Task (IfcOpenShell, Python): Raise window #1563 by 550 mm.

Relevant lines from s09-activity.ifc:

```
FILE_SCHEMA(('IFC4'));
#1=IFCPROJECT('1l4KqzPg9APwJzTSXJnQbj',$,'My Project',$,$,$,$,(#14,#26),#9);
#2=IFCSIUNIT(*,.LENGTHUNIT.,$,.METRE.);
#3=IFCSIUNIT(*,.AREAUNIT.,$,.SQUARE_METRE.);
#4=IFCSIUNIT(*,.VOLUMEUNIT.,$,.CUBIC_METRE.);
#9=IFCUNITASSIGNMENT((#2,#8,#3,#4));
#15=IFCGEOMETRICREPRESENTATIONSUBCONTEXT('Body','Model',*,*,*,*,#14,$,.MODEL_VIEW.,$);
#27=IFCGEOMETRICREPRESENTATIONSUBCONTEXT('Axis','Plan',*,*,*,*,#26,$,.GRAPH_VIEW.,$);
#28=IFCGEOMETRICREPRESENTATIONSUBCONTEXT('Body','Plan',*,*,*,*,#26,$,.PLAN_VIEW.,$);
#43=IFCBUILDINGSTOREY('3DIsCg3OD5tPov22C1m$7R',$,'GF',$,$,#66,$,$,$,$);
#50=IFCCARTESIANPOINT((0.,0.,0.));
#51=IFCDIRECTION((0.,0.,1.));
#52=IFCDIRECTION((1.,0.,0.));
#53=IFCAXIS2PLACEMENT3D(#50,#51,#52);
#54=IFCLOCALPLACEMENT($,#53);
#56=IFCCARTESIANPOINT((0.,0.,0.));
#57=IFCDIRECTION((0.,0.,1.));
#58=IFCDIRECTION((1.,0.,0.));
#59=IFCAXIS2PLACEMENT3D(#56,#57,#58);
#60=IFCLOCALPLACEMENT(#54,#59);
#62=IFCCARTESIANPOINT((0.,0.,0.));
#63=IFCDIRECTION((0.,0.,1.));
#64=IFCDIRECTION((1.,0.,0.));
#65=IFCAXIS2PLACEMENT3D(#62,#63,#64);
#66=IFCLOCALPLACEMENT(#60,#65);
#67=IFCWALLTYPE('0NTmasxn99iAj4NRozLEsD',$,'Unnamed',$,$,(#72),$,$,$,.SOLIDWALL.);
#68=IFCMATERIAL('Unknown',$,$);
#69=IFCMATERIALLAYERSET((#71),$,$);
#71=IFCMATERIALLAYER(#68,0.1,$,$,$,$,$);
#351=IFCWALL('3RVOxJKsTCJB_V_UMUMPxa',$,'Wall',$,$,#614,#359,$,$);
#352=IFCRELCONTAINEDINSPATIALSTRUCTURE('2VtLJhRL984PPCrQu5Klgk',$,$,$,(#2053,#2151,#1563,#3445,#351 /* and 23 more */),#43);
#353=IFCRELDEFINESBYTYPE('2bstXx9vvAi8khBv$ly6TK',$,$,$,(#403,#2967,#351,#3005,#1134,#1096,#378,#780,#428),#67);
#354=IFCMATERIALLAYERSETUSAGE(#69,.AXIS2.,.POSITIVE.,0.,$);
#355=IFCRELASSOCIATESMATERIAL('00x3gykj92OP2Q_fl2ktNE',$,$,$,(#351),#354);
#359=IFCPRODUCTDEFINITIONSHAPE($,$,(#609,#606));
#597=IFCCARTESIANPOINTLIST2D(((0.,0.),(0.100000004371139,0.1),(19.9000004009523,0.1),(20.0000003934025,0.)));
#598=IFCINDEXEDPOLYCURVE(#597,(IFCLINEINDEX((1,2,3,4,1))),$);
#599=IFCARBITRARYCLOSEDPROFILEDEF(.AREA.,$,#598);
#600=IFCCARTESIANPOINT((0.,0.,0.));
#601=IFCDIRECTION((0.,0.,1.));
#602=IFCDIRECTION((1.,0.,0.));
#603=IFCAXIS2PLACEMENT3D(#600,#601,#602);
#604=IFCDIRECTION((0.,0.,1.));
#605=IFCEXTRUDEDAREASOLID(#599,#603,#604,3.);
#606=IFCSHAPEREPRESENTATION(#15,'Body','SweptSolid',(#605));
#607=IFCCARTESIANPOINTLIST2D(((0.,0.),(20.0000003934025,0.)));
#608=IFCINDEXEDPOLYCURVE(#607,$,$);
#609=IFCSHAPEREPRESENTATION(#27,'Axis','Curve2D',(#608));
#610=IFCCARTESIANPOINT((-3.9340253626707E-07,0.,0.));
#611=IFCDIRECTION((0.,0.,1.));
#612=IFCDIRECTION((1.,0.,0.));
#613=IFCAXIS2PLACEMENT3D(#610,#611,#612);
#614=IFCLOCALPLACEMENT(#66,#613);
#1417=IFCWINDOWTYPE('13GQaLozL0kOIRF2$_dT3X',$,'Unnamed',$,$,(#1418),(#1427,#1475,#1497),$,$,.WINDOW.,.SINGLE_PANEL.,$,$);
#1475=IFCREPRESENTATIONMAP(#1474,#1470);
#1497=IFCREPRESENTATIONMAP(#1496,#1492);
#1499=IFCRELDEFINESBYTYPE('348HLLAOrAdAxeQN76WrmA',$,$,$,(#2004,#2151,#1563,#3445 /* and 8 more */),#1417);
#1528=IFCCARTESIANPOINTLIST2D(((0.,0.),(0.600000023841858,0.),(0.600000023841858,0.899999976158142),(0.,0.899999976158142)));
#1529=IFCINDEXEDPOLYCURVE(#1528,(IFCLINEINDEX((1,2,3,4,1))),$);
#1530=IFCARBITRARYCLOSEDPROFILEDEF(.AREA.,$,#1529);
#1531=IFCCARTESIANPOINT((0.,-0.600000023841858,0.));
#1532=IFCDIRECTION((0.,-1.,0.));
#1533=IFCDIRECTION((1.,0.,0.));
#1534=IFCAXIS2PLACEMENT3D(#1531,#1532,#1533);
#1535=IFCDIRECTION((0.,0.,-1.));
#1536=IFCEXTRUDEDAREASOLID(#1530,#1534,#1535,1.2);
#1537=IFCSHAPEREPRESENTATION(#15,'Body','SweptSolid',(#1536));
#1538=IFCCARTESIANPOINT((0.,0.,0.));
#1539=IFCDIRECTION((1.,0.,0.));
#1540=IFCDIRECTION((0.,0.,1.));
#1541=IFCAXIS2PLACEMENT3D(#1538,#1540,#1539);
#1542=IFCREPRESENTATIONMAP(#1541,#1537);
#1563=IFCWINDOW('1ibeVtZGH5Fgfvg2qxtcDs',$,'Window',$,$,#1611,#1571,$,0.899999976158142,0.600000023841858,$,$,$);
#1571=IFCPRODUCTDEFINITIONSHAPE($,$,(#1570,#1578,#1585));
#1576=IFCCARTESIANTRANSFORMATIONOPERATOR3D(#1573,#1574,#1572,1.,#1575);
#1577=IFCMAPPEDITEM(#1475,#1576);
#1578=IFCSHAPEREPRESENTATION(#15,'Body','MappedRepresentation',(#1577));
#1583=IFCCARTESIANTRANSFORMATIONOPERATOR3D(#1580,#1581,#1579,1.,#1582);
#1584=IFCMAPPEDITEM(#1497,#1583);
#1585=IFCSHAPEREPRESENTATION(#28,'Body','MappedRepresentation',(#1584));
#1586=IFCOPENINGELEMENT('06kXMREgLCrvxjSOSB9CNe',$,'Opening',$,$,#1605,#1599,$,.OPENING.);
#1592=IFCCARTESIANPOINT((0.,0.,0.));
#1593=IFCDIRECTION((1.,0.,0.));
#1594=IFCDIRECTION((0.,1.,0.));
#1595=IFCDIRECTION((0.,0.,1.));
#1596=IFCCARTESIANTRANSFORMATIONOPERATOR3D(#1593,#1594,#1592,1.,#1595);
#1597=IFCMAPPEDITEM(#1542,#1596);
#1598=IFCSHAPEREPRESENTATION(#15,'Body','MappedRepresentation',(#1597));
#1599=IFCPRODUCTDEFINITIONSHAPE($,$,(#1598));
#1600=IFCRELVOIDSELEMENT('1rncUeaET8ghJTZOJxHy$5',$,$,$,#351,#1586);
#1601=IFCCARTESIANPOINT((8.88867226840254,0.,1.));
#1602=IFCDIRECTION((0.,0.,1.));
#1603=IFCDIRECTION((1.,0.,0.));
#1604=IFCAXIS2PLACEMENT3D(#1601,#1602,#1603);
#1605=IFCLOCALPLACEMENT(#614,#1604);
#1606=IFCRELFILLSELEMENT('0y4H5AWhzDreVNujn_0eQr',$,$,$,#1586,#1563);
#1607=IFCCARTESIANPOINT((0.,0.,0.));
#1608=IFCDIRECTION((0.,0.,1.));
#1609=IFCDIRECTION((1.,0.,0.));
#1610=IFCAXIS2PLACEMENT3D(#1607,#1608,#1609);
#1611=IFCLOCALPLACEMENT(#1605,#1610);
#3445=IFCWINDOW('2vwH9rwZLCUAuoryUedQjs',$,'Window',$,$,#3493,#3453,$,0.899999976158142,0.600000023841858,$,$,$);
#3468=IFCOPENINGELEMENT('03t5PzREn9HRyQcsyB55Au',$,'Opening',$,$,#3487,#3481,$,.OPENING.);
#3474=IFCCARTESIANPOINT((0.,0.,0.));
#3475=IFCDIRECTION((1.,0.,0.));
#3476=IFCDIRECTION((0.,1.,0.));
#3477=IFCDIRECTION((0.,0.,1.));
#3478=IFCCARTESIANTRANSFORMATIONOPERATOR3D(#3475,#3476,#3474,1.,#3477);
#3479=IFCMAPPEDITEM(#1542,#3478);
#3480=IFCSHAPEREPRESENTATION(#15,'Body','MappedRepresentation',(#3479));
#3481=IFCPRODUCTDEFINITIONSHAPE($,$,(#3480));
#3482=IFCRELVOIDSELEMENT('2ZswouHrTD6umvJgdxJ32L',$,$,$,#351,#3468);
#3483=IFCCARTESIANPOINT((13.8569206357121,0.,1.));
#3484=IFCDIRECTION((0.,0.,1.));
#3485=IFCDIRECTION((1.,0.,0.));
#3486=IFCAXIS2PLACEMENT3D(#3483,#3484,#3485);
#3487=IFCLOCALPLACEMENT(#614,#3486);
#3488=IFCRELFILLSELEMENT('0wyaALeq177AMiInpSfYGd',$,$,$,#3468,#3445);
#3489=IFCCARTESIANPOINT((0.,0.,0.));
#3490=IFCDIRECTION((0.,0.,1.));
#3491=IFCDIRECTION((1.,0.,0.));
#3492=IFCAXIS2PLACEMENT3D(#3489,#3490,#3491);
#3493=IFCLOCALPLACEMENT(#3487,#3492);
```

```python
import numpy as np
import ifcopenshell
import ifcopenshell.api.geometry
import ifcopenshell.util.placement
import ifcopenshell.util.unit

model = ifcopenshell.open("s09-activity.ifc")
unit_scale = ifcopenshell.util.unit.calculate_unit_scale(model)

window = model.by_guid("1ibeVtZGH5Fgfvg2qxtcDs")
opening = window.FillsVoids[0].RelatingOpeningElement
dz = 0.55 / unit_scale

shift = np.array([0.0, 0.0, dz])
# The window is placed relative to its opening, so it follows when the opening moves.
matrix = ifcopenshell.util.placement.get_local_placement(opening.ObjectPlacement)
matrix[:3, 3] += shift
ifcopenshell.api.geometry.edit_object_placement(
    model, product=opening, matrix=matrix, is_si=False, should_transform_children=True
)

print(f"moved by {dz * unit_scale:+.3f} m")

model.write("s09-activity_v2.ifc")
```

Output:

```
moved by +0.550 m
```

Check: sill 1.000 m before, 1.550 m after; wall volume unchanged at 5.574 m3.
